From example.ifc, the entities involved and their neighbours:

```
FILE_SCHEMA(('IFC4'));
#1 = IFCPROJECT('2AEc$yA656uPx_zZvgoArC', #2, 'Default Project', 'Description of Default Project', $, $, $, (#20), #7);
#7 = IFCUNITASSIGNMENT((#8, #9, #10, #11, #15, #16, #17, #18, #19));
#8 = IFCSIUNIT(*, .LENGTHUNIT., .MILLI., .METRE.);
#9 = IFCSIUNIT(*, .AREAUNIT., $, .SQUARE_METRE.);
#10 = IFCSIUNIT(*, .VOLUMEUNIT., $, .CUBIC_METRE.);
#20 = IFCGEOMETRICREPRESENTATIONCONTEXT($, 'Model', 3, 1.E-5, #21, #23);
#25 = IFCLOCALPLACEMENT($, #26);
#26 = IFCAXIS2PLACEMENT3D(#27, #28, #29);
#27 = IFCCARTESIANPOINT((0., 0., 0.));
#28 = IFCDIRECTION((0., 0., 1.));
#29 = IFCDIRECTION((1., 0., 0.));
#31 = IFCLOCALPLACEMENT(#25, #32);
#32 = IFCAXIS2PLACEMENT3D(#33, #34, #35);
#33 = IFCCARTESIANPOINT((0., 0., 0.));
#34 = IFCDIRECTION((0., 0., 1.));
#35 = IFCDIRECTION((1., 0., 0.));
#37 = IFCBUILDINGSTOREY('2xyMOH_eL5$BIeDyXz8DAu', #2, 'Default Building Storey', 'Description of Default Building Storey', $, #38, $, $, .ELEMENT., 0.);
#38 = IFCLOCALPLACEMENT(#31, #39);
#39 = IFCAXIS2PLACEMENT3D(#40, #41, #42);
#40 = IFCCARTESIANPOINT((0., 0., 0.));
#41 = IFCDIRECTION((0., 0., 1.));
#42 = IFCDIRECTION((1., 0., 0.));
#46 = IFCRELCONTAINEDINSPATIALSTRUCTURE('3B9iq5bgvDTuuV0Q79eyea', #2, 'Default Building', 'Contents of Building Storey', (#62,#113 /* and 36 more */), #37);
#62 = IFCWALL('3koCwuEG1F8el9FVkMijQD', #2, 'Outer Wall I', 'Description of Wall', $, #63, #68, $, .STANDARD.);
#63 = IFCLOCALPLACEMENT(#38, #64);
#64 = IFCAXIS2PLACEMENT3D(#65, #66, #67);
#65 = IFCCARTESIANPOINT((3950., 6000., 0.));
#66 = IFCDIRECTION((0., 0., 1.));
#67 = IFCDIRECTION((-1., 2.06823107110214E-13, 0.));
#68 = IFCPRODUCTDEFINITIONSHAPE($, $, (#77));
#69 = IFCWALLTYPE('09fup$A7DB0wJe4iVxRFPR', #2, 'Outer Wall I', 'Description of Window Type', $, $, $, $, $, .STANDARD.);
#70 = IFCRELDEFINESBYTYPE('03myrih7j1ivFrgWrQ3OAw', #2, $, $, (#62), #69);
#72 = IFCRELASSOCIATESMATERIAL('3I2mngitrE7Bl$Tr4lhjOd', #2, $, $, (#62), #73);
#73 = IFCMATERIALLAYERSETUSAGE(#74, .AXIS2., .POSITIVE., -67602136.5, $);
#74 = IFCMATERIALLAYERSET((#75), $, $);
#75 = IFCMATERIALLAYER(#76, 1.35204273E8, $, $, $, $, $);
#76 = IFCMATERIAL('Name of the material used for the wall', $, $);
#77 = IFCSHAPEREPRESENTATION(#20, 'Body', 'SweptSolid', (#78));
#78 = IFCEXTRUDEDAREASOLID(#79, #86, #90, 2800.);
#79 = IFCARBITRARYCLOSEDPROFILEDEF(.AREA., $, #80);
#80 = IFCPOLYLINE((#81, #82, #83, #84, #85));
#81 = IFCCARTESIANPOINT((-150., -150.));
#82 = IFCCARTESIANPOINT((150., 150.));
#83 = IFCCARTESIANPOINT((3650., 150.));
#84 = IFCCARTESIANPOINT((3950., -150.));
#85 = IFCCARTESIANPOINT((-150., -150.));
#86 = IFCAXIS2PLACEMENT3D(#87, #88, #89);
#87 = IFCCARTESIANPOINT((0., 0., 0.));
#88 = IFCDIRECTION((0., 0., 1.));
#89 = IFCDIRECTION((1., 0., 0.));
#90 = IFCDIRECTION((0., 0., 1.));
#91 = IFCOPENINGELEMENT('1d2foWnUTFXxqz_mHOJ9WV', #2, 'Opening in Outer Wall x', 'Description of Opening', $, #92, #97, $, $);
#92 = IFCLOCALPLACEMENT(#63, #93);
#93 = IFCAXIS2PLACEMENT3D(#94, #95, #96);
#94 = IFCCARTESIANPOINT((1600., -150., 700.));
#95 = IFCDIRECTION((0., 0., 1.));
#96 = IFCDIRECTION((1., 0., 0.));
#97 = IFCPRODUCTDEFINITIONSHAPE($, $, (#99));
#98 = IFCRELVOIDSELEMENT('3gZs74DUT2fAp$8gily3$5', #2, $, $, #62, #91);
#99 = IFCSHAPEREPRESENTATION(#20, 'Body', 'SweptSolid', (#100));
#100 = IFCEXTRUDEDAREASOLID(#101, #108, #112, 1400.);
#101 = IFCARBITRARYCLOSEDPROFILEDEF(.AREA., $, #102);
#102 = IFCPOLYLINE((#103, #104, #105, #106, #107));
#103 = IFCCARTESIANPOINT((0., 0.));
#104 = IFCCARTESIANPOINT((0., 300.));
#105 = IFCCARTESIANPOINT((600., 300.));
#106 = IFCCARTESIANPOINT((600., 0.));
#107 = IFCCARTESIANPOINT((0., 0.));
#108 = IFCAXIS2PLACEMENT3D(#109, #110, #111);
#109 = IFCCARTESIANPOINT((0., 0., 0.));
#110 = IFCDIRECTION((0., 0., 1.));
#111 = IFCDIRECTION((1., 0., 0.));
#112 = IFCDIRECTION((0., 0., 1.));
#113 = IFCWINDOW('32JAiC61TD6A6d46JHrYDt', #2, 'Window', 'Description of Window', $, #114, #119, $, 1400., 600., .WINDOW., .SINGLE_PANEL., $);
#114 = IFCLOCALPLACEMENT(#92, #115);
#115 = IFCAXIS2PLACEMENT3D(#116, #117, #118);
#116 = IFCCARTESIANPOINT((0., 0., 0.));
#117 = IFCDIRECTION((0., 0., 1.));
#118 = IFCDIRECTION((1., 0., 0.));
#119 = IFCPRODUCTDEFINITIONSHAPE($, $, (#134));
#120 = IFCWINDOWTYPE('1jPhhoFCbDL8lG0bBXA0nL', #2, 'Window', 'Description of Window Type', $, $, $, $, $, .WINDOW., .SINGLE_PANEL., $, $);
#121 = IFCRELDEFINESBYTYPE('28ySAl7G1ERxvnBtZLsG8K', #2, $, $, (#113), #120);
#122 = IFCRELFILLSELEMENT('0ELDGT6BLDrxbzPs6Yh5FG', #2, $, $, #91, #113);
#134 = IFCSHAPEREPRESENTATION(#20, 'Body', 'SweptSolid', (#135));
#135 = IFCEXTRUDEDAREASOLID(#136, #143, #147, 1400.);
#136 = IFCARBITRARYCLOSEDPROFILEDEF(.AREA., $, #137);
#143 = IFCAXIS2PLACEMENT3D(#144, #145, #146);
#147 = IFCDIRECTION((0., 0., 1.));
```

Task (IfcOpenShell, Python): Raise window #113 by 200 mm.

```python
import numpy as np
import ifcopenshell
import ifcopenshell.api.geometry
import ifcopenshell.util.placement
import ifcopenshell.util.unit

model = ifcopenshell.open("example.ifc")
unit_scale = ifcopenshell.util.unit.calculate_unit_scale(model)

window = model.by_id(113)
opening = window.FillsVoids[0].RelatingOpeningElement
dz = 0.2 / unit_scale

shift = np.array([0.0, 0.0, dz])
# The window is placed relative to its opening, so it follows when the opening moves.
matrix = ifcopenshell.util.placement.get_local_placement(opening.ObjectPlacement)
matrix[:3, 3] += shift
ifcopenshell.api.geometry.edit_object_placement(
    model, product=opening, matrix=matrix, is_si=False, should_transform_children=True
)

print(f"moved by {dz * unit_scale:+.3f} m")

model.write("example-out.ifc")
```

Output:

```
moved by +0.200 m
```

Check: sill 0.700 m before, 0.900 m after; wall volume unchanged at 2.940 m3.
